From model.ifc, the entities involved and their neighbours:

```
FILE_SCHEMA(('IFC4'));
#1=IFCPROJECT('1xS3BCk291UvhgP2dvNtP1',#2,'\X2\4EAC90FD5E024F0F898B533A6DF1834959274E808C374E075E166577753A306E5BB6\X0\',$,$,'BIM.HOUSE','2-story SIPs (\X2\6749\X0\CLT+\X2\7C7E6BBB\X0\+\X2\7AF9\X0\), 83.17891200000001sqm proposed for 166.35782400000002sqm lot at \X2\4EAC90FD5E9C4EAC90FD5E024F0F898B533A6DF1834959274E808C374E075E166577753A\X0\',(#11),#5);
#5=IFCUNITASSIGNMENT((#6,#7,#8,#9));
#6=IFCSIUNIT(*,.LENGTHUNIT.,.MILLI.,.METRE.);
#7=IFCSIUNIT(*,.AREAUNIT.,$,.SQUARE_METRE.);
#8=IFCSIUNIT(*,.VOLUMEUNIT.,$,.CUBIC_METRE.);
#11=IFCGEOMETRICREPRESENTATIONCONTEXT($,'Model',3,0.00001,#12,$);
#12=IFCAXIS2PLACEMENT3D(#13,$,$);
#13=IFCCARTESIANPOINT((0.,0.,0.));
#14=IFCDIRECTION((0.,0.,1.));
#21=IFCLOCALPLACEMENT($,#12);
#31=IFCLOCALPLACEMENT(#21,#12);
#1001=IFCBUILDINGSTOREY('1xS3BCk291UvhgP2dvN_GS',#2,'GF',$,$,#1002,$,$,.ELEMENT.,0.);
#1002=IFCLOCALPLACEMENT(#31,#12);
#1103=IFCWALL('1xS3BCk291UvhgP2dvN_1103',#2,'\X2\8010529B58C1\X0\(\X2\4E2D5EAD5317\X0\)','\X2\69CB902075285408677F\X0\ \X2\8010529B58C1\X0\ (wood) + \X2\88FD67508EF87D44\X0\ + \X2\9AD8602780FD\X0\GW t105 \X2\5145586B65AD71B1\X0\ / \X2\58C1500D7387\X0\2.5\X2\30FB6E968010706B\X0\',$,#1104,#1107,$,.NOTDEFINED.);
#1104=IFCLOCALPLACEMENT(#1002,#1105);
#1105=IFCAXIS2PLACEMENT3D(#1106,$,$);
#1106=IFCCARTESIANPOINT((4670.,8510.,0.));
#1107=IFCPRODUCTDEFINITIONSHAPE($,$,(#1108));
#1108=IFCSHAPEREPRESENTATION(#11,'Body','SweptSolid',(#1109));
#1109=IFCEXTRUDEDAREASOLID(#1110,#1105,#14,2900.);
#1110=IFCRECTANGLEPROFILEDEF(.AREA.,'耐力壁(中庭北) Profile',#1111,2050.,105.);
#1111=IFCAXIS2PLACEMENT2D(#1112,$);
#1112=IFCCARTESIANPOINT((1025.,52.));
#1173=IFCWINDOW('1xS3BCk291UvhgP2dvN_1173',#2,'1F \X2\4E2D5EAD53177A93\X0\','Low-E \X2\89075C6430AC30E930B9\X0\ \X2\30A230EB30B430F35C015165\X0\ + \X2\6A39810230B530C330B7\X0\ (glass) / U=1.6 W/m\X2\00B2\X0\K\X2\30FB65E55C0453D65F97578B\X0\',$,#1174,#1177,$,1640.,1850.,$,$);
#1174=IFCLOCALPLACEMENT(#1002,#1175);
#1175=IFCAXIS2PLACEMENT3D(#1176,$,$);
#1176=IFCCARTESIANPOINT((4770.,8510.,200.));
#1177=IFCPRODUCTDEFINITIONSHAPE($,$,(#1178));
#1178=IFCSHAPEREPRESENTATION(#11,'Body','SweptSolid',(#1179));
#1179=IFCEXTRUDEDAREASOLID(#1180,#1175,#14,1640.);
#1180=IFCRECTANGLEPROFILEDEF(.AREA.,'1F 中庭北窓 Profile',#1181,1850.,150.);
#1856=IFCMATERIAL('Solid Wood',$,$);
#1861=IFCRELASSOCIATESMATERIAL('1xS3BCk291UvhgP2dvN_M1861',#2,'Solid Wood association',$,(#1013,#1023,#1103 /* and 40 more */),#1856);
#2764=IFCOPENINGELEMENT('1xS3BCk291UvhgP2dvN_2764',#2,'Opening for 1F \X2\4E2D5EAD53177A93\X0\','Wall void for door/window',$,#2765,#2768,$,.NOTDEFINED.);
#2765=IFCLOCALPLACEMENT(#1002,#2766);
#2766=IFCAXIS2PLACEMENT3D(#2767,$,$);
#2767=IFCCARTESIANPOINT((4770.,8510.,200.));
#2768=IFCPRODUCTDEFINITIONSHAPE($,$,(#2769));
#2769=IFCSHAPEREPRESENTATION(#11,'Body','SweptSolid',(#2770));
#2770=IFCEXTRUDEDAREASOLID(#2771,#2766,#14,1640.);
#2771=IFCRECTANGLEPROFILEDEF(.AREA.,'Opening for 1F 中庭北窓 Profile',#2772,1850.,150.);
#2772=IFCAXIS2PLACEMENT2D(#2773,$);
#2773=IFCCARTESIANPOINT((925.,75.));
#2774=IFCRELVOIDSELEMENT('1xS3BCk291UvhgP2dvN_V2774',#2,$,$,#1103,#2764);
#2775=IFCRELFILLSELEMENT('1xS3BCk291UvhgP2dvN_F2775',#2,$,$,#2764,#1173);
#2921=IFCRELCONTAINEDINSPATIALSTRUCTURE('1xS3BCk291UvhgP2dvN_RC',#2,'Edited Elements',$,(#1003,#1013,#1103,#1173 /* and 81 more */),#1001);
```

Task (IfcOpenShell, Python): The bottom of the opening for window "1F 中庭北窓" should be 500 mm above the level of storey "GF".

```python
import numpy as np
import ifcopenshell
import ifcopenshell.api.geometry
import ifcopenshell.geom
import ifcopenshell.util.element
import ifcopenshell.util.placement
import ifcopenshell.util.shape
import ifcopenshell.util.unit

model = ifcopenshell.open("model.ifc")
unit_scale = ifcopenshell.util.unit.calculate_unit_scale(model)

window = model.by_guid("1xS3BCk291UvhgP2dvN_1173")
opening = window.FillsVoids[0].RelatingOpeningElement
storey = ifcopenshell.util.element.get_container(window, ifc_class="IfcBuildingStorey")
level = ifcopenshell.util.placement.get_local_placement(storey.ObjectPlacement)[2, 3]

# The opening's origin need not be at the sill, so measure its lowest point.
shape = ifcopenshell.geom.create_shape(ifcopenshell.geom.settings(), opening)
bottom = ifcopenshell.util.shape.get_shape_bottom_elevation(shape, shape.geometry) / unit_scale
dz = level + 0.5 / unit_scale - bottom

shift = np.array([0.0, 0.0, dz])
# The window is not placed relative to its opening, so move both.
for product in (opening, window):
    matrix = ifcopenshell.util.placement.get_local_placement(product.ObjectPlacement)
    matrix[:3, 3] += shift
    ifcopenshell.api.geometry.edit_object_placement(model, product=product, matrix=matrix, is_si=False)

print(f"moved by {dz * unit_scale:+.3f} m")

model.write("model_v2.ifc")
```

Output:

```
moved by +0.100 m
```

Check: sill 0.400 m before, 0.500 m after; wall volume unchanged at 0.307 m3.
